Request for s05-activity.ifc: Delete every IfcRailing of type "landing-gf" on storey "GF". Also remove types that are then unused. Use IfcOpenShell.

First a look at what the model holds.

```python
import ifcopenshell
import ifcopenshell.util.element

model = ifcopenshell.open("s05-activity.ifc")
print(model.schema)
storey = next(s for s in model.by_type("IfcBuildingStorey") if s.Name == "GF")
railings = [e for e in ifcopenshell.util.element.get_decomposition(storey) if e.is_a("IfcRailing")]
seen = {}
for e in railings:
    element_type = ifcopenshell.util.element.get_type(e)
    name = element_type.Name if element_type not in (None, e) else None
    seen[name] = seen.get(name, 0) + 1
for name, count in sorted(seen.items(), key=str):
    print(count, "x", name)
```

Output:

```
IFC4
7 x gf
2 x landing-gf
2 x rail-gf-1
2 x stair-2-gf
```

```python
import ifcopenshell
import ifcopenshell.api.root
import ifcopenshell.util.element

model = ifcopenshell.open("s05-activity.ifc")

storey = next(s for s in model.by_type("IfcBuildingStorey") if s.Name == "GF")
railings = [e for e in ifcopenshell.util.element.get_decomposition(storey) if e.is_a("IfcRailing")]
targets = [e for e in railings if (t := ifcopenshell.util.element.get_type(e)) not in (None, e) and t.Name == "landing-gf"]
types = {ifcopenshell.util.element.get_type(e) for e in targets} - {None, *targets}

for e in targets:
    ifcopenshell.api.root.remove_product(model, product=e)
print(len(targets), "removed")

unused = [t for t in types if not ifcopenshell.util.element.get_types(t)]
for t in unused:
    ifcopenshell.api.root.remove_product(model, product=t)
print(len(unused), "unused types removed")

model.write("s05-activity_rev.ifc")
```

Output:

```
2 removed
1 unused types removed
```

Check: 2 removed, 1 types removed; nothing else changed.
